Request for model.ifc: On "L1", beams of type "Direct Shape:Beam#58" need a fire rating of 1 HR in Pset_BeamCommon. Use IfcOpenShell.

First a look at what the model holds.

```python
import ifcopenshell
import ifcopenshell.util.element

model = ifcopenshell.open("model.ifc")
print(model.schema)
storey = next(s for s in model.by_type("IfcBuildingStorey") if s.Name == "L1")
beams = [e for e in ifcopenshell.util.element.get_decomposition(storey) if e.is_a("IfcBeam")]
seen = {}
for e in beams:
    element_type = ifcopenshell.util.element.get_type(e)
    key = (element_type.Name if element_type != e and element_type else None, ifcopenshell.util.element.get_pset(e, "Pset_BeamCommon", "FireRating"))
    seen[key] = seen.get(key, 0) + 1
for (name, value), count in sorted(seen.items(), key=str):
    print(count, "x", name, "|", value)
```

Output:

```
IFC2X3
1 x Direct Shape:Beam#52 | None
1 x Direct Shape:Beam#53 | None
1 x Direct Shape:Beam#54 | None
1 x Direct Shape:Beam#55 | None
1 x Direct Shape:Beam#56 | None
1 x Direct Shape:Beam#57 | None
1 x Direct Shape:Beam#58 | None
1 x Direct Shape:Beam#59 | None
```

```python
import ifcopenshell
import ifcopenshell.api.pset
import ifcopenshell.util.element

model = ifcopenshell.open("model.ifc")

storey = next(s for s in model.by_type("IfcBuildingStorey") if s.Name == "L1")
beams = [e for e in ifcopenshell.util.element.get_decomposition(storey) if e.is_a("IfcBeam")]

count = 0
for e in beams:
    element_type = ifcopenshell.util.element.get_type(e)
    if element_type in (None, e) or element_type.Name != "Direct Shape:Beam#58":
        continue
    # add_pset returns the element's existing set when there is one.
    pset = ifcopenshell.api.pset.add_pset(model, product=e, name="Pset_BeamCommon")
    ifcopenshell.api.pset.edit_pset(model, pset=pset, properties={"FireRating": "1 HR"})
    count += 1

print(count, "beams updated")

model.write("model_rev.ifc")
```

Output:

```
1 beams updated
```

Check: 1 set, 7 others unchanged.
